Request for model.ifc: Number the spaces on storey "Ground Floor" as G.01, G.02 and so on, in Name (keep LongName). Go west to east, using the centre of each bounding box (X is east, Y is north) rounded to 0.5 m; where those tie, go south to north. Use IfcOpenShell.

First a look at what the model holds.

```python
import ifcopenshell
import ifcopenshell.util.element
import ifcopenshell.util.placement

model = ifcopenshell.open("model.ifc")
print(model.schema)
storey = next(s for s in model.by_type("IfcBuildingStorey") if s.Name == "Ground Floor")
spaces = [e for e in ifcopenshell.util.element.get_decomposition(storey) if e.is_a("IfcSpace")]
for e in sorted(spaces, key=lambda e: e.id()):
    origin = ifcopenshell.util.placement.get_local_placement(e.ObjectPlacement)[:3, 3]
    print(e.id(), e.Name, e.LongName, origin.round(2) + 0.0, sep=" | ")
```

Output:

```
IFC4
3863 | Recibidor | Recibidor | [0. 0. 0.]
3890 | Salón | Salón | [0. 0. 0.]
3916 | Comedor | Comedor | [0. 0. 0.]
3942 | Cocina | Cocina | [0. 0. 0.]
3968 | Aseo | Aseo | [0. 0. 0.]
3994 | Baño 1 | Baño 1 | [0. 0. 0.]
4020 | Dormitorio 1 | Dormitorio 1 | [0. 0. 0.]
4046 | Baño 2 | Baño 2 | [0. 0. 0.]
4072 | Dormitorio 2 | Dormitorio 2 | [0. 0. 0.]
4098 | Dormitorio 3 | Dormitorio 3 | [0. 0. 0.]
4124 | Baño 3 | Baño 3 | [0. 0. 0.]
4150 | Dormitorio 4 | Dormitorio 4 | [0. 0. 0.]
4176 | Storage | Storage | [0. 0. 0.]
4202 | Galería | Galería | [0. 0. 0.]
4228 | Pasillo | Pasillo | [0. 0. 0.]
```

```python
import ifcopenshell
import ifcopenshell.geom
import ifcopenshell.util.element
import ifcopenshell.util.shape

model = ifcopenshell.open("model.ifc")
settings = ifcopenshell.geom.settings()
settings.set("use-world-coords", True)


def centre(element):
    shape = ifcopenshell.geom.create_shape(settings, element)
    return ifcopenshell.util.shape.get_bbox_centroid(shape.geometry)


storey = next(s for s in model.by_type("IfcBuildingStorey") if s.Name == "Ground Floor")
spaces = [e for e in ifcopenshell.util.element.get_decomposition(storey) if e.is_a("IfcSpace")]

# Insertion points can sit at a corner or the storey origin, so sort by the geometry (in metres).
centres = {e: centre(e) for e in spaces}
spaces.sort(key=lambda e: (round(centres[e][0] / 0.5), centres[e][1]))

for i, e in enumerate(spaces, start=1):
    number = f"G.{i:02d}"
    e.Name = number
    print(e.id(), number)

model.write("model_edited.ifc")
```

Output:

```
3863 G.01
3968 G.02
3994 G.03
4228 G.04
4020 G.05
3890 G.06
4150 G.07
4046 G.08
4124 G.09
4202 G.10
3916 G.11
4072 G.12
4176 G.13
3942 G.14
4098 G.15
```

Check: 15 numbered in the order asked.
